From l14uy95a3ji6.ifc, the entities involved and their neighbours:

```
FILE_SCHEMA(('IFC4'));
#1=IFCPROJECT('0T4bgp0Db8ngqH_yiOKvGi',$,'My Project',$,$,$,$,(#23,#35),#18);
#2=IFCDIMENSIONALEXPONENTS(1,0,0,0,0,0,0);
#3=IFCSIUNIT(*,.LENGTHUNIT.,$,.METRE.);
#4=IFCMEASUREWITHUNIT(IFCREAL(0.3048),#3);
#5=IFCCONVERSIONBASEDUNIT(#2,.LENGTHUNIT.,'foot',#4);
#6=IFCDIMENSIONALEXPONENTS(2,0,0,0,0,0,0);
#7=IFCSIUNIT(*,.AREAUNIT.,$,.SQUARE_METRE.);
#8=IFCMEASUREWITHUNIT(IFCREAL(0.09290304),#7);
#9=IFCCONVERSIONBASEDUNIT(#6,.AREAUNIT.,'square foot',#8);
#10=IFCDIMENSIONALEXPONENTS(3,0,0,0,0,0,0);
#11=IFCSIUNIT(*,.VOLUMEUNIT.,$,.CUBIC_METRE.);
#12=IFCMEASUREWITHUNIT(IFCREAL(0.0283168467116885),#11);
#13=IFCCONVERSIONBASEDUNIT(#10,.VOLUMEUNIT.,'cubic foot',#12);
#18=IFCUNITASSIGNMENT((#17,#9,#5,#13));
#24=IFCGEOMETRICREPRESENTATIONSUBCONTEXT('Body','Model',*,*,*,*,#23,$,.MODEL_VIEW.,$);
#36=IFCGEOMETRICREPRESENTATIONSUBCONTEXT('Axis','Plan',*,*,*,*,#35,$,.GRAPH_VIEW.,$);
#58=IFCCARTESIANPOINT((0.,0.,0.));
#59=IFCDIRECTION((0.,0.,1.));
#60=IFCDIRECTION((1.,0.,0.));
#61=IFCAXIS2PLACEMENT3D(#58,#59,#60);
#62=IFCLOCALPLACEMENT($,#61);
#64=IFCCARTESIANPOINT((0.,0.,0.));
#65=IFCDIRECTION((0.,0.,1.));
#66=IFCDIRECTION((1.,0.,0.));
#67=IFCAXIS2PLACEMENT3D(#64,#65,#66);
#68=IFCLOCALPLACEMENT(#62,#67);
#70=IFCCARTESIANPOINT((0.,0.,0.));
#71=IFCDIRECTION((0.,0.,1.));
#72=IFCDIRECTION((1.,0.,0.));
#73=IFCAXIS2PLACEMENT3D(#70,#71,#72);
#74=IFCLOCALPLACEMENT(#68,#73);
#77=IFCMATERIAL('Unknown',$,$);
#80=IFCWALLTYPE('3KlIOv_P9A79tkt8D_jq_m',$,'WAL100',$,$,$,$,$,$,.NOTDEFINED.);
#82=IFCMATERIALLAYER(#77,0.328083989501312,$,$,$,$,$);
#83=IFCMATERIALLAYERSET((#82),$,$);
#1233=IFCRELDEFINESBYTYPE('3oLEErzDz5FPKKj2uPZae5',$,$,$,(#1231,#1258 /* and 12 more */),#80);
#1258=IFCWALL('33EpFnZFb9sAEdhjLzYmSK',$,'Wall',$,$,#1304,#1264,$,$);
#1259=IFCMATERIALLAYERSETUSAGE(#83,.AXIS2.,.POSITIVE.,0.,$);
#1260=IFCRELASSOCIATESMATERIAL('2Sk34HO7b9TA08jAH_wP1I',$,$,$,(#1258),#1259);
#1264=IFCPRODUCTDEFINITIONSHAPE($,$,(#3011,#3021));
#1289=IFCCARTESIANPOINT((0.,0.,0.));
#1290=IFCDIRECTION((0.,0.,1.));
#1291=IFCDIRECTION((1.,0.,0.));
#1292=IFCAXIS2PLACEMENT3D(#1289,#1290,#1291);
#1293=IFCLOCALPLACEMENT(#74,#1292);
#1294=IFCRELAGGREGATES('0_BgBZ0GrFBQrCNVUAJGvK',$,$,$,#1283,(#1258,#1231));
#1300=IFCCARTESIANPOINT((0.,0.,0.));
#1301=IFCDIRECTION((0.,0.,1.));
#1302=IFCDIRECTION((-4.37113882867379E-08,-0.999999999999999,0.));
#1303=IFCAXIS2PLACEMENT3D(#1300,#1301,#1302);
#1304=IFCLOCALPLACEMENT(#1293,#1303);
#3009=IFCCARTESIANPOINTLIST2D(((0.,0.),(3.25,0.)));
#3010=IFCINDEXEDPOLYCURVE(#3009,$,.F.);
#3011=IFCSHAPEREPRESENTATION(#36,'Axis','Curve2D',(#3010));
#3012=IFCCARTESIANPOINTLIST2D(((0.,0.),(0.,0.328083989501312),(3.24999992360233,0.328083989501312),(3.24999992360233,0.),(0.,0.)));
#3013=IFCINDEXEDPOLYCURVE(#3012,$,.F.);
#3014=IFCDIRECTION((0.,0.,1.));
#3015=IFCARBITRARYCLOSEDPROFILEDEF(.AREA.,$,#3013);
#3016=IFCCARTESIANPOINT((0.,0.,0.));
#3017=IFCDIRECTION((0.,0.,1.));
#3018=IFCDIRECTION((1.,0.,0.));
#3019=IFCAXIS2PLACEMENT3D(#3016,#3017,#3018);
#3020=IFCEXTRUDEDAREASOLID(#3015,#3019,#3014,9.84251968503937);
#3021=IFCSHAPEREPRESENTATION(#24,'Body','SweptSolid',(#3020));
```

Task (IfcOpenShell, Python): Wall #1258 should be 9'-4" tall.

```python
import ifcopenshell
import ifcopenshell.geom
import ifcopenshell.util.representation
import ifcopenshell.util.shape
import ifcopenshell.util.unit

model = ifcopenshell.open("l14uy95a3ji6.ifc")
unit_scale = ifcopenshell.util.unit.calculate_unit_scale(model)
settings = ifcopenshell.geom.settings()


def volume(element):
    """Net volume in cubic metres, openings subtracted."""
    shape = ifcopenshell.geom.create_shape(settings, element)
    return ifcopenshell.util.shape.get_volume(shape.geometry)


wall = model.by_id(1258)
before = volume(wall)

body = ifcopenshell.util.representation.get_representation(wall, "Model", "Body")
solid = body.Items[0]
old_height = solid.Depth
solid.Depth = 112 * 0.0254 / unit_scale
after = volume(wall)

print(f"height {old_height:g} -> {solid.Depth:g}, volume {before:.3f} -> {after:.3f} m3")

model.write("l14uy95a3ji6_edited.ifc")
```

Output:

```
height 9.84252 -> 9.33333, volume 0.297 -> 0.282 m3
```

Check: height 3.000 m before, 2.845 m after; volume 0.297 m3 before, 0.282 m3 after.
